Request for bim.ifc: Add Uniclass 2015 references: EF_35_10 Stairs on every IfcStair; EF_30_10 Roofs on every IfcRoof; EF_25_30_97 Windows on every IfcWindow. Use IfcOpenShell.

First a look at what the model holds.

```python
import ifcopenshell

model = ifcopenshell.open("bim.ifc")
print(model.schema)
print("classifications:", [c.Name for c in model.by_type("IfcClassification")])
for ifc_class in ("IfcDoor", "IfcRoof", "IfcStair", "IfcWall", "IfcWindow"):
    print(ifc_class, len(model.by_type(ifc_class)))
```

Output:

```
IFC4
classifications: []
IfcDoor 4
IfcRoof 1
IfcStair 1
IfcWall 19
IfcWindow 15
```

```python
import ifcopenshell
import ifcopenshell.api.classification

model = ifcopenshell.open("bim.ifc")

system = ifcopenshell.api.classification.add_classification(model, classification="Uniclass 2015")

codes = {
    "IfcStair": ("EF_35_10", "Stairs"),
    "IfcRoof": ("EF_30_10", "Roofs"),
    "IfcWindow": ("EF_25_30_97", "Windows"),
}
for ifc_class, (code, name) in codes.items():
    products = model.by_type(ifc_class)
    ifcopenshell.api.classification.add_reference(
        model, products=products, classification=system, identification=code, name=name
    )
    print(code, len(products))

model.write("bim_updated.ifc")
```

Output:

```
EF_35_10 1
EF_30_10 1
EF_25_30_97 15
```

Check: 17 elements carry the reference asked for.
